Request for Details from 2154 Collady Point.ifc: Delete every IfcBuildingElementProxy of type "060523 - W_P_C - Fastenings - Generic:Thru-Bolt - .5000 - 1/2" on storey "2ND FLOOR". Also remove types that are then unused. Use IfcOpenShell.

First a look at what the model holds.

```python
import ifcopenshell
import ifcopenshell.util.element

model = ifcopenshell.open("Details from 2154 Collady Point.ifc")
print(model.schema)
storey = next(s for s in model.by_type("IfcBuildingStorey") if s.Name == "2ND FLOOR")
proxies = [e for e in ifcopenshell.util.element.get_decomposition(storey) if e.is_a("IfcBuildingElementProxy")]
seen = {}
for e in proxies:
    element_type = ifcopenshell.util.element.get_type(e)
    name = element_type.Name if element_type not in (None, e) else None
    seen[name] = seen.get(name, 0) + 1
for name, count in sorted(seen.items(), key=str):
    print(count, "x", name)
```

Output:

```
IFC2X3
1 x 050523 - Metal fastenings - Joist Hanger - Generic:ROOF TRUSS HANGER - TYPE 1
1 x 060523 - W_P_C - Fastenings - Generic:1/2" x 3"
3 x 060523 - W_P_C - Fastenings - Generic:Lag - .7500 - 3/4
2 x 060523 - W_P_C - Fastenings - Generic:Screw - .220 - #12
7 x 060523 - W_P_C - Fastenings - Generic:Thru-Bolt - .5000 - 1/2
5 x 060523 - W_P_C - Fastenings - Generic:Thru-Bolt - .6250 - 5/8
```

```python
import ifcopenshell
import ifcopenshell.api.root
import ifcopenshell.util.element

model = ifcopenshell.open("Details from 2154 Collady Point.ifc")

storey = next(s for s in model.by_type("IfcBuildingStorey") if s.Name == "2ND FLOOR")
proxies = [e for e in ifcopenshell.util.element.get_decomposition(storey) if e.is_a("IfcBuildingElementProxy")]
targets = [e for e in proxies if (t := ifcopenshell.util.element.get_type(e)) not in (None, e) and t.Name == "060523 - W_P_C - Fastenings - Generic:Thru-Bolt - .5000 - 1/2"]
types = {ifcopenshell.util.element.get_type(e) for e in targets} - {None, *targets}

for e in targets:
    ifcopenshell.api.root.remove_product(model, product=e)
print(len(targets), "removed")

unused = [t for t in types if not ifcopenshell.util.element.get_types(t)]
for t in unused:
    ifcopenshell.api.root.remove_product(model, product=t)
print(len(unused), "unused types removed")

model.write("Details from 2154 Collady Point_v2.ifc")
```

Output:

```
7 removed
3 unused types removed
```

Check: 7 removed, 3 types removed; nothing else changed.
